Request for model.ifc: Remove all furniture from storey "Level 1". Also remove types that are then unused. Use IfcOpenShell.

First a look at what the model holds.

```python
import ifcopenshell
import ifcopenshell.util.element

model = ifcopenshell.open("model.ifc")
print(model.schema)
storey = next(s for s in model.by_type("IfcBuildingStorey") if s.Name == "Level 1")
furniture = [e for e in ifcopenshell.util.element.get_decomposition(storey) if e.is_a("IfcFurnishingElement")]
seen = {}
for e in furniture:
    element_type = ifcopenshell.util.element.get_type(e)
    name = element_type.Name if element_type not in (None, e) else None
    seen[name] = seen.get(name, 0) + 1
for name, count in sorted(seen.items(), key=str):
    print(count, "x", name)
```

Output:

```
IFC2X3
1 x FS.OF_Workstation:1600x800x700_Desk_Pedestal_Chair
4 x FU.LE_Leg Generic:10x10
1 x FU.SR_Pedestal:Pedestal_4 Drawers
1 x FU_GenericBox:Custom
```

```python
import ifcopenshell
import ifcopenshell.api.root
import ifcopenshell.util.element

model = ifcopenshell.open("model.ifc")

storey = next(s for s in model.by_type("IfcBuildingStorey") if s.Name == "Level 1")
furniture = [e for e in ifcopenshell.util.element.get_decomposition(storey) if e.is_a("IfcFurnishingElement")]
types = {ifcopenshell.util.element.get_type(e) for e in furniture} - {None, *furniture}

for e in furniture:
    ifcopenshell.api.root.remove_product(model, product=e)
print(len(furniture), "removed")

unused = [t for t in types if not ifcopenshell.util.element.get_types(t)]
for t in unused:
    ifcopenshell.api.root.remove_product(model, product=t)
print(len(unused), "unused types removed")

model.write("model_updated.ifc")
```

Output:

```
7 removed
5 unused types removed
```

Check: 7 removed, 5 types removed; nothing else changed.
